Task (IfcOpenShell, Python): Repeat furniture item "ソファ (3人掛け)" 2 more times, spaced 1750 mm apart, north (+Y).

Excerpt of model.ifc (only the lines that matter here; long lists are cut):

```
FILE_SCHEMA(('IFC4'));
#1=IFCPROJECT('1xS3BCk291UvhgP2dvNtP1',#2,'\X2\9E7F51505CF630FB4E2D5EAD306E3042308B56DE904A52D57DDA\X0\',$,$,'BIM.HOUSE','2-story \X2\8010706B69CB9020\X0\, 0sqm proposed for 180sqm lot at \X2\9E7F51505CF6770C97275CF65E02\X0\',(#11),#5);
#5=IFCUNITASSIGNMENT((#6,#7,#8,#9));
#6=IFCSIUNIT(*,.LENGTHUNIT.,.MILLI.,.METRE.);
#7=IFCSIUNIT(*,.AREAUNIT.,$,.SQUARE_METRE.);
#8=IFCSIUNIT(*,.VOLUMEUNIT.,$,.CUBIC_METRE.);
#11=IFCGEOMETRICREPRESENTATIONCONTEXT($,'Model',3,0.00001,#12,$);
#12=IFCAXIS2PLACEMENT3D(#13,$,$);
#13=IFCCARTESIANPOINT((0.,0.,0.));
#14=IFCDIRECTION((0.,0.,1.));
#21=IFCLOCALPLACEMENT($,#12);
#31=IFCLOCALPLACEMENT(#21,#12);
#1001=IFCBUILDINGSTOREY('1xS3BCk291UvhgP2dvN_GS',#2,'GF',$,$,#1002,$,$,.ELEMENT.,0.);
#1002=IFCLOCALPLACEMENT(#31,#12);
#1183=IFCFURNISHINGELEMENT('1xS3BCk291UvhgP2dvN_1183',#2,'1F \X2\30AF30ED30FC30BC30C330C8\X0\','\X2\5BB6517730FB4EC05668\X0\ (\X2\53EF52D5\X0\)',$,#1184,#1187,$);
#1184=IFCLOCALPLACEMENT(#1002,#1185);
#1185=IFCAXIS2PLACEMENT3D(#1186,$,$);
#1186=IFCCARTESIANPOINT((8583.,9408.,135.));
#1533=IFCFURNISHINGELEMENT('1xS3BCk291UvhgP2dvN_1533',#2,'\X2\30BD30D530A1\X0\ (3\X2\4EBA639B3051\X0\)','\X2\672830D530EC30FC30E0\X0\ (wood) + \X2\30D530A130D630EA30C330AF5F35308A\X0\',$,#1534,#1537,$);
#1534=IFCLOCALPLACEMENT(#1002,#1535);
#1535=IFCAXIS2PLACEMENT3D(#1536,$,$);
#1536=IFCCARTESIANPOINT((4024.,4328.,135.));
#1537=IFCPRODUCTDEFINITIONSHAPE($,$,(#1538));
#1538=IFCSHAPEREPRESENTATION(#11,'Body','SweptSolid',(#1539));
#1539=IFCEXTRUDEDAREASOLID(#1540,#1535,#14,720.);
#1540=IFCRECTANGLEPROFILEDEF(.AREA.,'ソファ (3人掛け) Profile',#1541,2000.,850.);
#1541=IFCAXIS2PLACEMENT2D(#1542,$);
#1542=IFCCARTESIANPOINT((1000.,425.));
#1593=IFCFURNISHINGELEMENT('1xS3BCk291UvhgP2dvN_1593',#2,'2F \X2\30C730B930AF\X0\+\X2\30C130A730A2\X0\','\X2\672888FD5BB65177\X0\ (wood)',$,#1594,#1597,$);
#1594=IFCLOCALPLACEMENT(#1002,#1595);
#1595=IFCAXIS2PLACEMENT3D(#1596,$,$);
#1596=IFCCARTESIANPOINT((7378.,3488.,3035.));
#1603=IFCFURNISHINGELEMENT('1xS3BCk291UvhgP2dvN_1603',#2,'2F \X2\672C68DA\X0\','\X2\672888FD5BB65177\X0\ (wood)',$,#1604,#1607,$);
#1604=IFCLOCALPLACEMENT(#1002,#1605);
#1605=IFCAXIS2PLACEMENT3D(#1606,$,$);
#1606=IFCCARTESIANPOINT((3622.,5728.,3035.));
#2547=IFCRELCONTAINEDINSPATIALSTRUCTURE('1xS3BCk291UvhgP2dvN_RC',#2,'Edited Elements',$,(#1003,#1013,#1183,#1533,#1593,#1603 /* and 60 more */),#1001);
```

```python
import numpy as np
import ifcopenshell
import ifcopenshell.api.geometry
import ifcopenshell.api.root
import ifcopenshell.util.element
import ifcopenshell.util.placement
import ifcopenshell.util.unit

model = ifcopenshell.open("model.ifc")
unit_scale = ifcopenshell.util.unit.calculate_unit_scale(model)


def reuse_history(source, copy):
    """copy_class also copies each property set's owner history, people and application; keep the originals."""
    for rel in copy.IsDefinedBy:
        if rel.is_a("IfcRelDefinesByProperties") and (history := rel.RelatingPropertyDefinition.OwnerHistory):
            rel.RelatingPropertyDefinition.OwnerHistory = source.OwnerHistory
            ifcopenshell.util.element.remove_deep2(model, history)


source = model.by_guid("1xS3BCk291UvhgP2dvN_1533")
base = ifcopenshell.util.placement.get_local_placement(source.ObjectPlacement)
step = np.array([0.0, 1.0, 0.0]) * 1.75 / unit_scale

for i in range(1, 3):
    copy = ifcopenshell.api.root.copy_class(model, product=source)
    copy.Representation = ifcopenshell.util.element.copy_deep(
        model, source.Representation, exclude=["IfcGeometricRepresentationContext", "IfcRepresentationMap"]
    )
    reuse_history(source, copy)
    matrix = base.copy()
    matrix[:3, 3] += i * step
    print("added at", matrix[:3, 3].round(3) + 0.0)
    ifcopenshell.api.geometry.edit_object_placement(model, product=copy, matrix=matrix, is_si=False)

model.write("model_rev.ifc")
```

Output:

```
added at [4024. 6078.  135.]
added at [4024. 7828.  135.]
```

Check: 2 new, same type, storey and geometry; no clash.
